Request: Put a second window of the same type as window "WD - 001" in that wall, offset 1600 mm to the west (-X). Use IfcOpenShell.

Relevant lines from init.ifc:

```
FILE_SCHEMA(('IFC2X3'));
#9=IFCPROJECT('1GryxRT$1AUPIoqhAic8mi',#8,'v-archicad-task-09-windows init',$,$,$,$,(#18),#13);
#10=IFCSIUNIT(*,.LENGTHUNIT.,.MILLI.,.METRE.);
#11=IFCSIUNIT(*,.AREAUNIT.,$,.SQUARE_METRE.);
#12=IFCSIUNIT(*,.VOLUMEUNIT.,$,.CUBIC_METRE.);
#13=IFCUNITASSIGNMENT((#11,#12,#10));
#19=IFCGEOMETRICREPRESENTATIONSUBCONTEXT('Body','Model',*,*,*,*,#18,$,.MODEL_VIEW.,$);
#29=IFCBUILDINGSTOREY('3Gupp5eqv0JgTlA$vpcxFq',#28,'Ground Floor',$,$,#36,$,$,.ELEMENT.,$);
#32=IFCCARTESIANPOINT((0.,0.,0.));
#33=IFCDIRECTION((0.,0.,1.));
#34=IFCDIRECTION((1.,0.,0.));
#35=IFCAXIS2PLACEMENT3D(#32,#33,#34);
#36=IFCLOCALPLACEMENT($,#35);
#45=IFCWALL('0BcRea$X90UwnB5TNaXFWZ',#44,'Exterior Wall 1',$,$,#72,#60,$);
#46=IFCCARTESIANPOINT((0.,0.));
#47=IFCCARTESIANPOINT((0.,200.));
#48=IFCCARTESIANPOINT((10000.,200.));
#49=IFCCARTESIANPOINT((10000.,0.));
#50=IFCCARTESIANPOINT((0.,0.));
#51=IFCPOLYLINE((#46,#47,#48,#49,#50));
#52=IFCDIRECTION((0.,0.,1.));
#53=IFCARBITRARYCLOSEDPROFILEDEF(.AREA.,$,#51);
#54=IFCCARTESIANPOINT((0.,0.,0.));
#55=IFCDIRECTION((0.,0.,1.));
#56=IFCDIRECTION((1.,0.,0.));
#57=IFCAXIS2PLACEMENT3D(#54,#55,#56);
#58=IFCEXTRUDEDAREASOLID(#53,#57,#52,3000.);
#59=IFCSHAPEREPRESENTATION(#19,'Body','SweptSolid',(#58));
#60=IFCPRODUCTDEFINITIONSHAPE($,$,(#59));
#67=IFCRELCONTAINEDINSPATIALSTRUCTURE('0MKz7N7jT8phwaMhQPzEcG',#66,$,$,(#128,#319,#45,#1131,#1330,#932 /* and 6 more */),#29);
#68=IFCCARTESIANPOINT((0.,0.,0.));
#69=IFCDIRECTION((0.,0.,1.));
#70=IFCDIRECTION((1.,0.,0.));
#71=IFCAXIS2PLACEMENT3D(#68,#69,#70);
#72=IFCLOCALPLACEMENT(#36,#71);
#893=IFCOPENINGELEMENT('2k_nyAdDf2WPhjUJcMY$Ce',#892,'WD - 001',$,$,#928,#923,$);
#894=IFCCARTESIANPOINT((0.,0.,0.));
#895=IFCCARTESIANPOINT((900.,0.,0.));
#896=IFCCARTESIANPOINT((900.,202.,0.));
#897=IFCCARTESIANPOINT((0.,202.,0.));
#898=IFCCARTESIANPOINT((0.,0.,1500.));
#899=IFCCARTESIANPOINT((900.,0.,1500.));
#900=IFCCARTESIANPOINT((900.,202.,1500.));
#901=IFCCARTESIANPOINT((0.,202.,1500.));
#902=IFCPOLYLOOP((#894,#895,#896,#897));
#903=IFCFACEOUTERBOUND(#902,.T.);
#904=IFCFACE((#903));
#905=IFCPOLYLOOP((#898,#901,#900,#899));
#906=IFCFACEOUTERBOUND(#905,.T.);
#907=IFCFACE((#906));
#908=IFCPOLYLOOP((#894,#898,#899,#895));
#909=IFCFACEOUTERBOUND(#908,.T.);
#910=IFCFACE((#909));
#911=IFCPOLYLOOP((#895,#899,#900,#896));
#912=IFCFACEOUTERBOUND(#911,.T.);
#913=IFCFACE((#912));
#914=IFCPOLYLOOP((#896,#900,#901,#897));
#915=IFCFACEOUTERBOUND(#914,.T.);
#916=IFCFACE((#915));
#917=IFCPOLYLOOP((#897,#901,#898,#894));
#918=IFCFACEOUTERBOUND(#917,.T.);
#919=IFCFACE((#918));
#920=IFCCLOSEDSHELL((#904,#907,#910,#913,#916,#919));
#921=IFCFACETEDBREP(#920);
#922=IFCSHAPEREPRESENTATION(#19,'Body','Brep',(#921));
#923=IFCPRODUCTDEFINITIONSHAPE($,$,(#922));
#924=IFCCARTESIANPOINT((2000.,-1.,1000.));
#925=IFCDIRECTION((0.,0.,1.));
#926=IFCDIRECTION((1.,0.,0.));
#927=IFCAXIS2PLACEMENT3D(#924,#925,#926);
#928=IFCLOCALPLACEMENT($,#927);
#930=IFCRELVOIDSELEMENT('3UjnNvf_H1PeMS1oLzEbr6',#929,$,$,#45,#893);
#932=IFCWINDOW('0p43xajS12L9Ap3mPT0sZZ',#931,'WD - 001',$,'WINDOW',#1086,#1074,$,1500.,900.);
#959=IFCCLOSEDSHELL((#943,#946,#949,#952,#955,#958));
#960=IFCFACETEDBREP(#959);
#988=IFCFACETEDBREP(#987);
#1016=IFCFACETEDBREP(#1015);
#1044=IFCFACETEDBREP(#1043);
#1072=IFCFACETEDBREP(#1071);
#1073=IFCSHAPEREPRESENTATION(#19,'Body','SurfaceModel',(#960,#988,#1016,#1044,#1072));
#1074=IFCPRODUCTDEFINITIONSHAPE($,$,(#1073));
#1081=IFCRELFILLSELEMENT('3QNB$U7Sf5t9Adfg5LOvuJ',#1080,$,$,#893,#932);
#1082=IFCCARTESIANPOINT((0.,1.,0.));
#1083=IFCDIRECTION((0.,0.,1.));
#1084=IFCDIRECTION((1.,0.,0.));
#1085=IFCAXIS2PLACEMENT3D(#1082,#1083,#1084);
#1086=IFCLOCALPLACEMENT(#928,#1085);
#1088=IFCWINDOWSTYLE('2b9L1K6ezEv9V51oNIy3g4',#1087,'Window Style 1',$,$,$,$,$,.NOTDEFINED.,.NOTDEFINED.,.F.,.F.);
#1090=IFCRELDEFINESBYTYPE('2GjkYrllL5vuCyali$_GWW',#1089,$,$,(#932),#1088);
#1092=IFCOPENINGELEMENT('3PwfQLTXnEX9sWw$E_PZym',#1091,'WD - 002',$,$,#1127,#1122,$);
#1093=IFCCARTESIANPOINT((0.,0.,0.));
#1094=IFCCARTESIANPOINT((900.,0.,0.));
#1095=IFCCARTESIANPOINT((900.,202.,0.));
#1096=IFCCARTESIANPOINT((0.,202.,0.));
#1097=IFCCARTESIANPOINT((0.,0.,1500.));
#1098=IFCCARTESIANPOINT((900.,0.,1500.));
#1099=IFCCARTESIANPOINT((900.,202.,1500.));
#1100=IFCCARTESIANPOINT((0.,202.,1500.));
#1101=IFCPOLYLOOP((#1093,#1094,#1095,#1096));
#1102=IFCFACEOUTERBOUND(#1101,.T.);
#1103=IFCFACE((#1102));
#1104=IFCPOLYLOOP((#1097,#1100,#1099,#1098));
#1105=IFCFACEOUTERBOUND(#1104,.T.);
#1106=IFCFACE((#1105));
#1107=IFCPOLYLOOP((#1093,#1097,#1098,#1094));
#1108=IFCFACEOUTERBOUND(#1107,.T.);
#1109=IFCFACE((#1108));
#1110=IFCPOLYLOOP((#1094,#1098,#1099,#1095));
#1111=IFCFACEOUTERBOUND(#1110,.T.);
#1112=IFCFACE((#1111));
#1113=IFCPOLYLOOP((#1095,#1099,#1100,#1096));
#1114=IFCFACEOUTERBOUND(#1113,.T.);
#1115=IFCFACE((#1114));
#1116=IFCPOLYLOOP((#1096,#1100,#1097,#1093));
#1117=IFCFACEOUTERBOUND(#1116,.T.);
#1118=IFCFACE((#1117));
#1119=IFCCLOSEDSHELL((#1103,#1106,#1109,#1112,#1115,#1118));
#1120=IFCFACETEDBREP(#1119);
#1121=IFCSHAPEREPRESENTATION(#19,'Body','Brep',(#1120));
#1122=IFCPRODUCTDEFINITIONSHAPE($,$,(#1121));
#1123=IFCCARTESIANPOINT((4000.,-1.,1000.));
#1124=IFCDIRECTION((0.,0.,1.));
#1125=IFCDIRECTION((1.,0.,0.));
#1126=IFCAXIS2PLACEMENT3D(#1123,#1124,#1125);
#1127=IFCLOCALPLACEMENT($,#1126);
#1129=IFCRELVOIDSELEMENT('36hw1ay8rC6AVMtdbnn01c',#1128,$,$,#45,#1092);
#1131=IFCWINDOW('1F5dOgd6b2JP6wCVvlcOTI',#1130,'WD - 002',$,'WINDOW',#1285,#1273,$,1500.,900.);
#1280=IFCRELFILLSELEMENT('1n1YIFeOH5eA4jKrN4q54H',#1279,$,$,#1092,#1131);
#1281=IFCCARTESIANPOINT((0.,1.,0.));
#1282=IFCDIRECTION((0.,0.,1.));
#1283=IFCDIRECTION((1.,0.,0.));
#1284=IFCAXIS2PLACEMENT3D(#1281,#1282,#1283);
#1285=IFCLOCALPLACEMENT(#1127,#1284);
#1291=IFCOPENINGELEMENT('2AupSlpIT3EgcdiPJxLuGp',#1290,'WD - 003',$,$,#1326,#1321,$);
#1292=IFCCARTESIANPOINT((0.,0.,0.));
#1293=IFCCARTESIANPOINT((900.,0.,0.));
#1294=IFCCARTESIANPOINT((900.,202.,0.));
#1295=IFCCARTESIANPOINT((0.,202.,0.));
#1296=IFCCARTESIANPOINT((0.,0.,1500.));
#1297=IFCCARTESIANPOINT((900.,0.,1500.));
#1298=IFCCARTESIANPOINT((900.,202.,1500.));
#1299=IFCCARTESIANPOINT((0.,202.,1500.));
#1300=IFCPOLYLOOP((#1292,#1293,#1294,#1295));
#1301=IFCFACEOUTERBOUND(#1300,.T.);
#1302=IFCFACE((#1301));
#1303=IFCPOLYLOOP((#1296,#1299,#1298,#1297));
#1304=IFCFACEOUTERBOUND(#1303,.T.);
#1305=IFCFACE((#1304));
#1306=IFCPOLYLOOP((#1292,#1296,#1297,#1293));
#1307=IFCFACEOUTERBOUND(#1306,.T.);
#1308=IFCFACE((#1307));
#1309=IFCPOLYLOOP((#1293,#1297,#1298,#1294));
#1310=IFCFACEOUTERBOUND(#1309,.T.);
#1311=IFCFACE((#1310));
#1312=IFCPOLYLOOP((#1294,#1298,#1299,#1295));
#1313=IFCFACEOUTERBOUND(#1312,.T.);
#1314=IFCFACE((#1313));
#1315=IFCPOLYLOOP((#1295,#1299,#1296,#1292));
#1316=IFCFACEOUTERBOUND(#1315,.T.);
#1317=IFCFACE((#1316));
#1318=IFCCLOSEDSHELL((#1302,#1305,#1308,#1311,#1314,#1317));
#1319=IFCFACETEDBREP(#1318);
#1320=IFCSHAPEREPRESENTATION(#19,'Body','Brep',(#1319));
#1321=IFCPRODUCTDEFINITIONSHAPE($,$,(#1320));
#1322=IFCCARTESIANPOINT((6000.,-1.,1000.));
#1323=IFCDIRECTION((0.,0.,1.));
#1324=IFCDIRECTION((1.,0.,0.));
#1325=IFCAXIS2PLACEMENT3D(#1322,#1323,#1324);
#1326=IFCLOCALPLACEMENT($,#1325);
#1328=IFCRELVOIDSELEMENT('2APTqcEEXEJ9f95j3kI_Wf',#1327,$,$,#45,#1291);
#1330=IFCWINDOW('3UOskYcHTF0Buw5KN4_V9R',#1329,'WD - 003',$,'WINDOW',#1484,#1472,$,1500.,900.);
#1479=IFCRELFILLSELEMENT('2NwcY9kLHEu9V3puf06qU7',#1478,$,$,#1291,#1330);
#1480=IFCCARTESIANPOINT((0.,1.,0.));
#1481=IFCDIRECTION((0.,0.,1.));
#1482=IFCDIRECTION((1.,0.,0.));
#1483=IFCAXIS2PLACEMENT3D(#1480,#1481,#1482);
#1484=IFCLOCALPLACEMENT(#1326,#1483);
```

```python
import ifcopenshell
import ifcopenshell.api.feature
import ifcopenshell.api.geometry
import ifcopenshell.api.root
import ifcopenshell.geom
import ifcopenshell.util.element
import ifcopenshell.util.placement
import ifcopenshell.util.shape
import ifcopenshell.util.unit

model = ifcopenshell.open("init.ifc")
unit_scale = ifcopenshell.util.unit.calculate_unit_scale(model)
settings = ifcopenshell.geom.settings()


def volume(element):
    """Net volume in cubic metres, openings subtracted."""
    shape = ifcopenshell.geom.create_shape(settings, element)
    return ifcopenshell.util.shape.get_volume(shape.geometry)


window = model.by_guid("0p43xajS12L9Ap3mPT0sZZ")
opening = window.FillsVoids[0].RelatingOpeningElement
wall = opening.VoidsElements[0].RelatingBuildingElement
before = volume(wall)
shift = ifcopenshell.util.placement.get_local_placement(wall.ObjectPlacement)[:3, 0] * -1.6 / unit_scale

# copy_class copies the void relationship, type, container and properties, but no geometry.
new_opening = ifcopenshell.api.root.copy_class(model, product=opening)
new_opening.Representation = ifcopenshell.util.element.copy_deep(
    model, opening.Representation, exclude=["IfcGeometricRepresentationContext", "IfcRepresentationMap"]
)
new_window = ifcopenshell.api.root.copy_class(model, product=window)
new_window.Representation = ifcopenshell.util.element.copy_deep(
    model, window.Representation, exclude=["IfcGeometricRepresentationContext", "IfcRepresentationMap"]
)
fills = ifcopenshell.api.feature.add_filling(model, opening=new_opening, element=new_window)
fills.OwnerHistory = new_window.OwnerHistory  # required in IFC2X3

for old, new in ((opening, new_opening), (window, new_window)):
    matrix = ifcopenshell.util.placement.get_local_placement(old.ObjectPlacement)
    matrix[:3, 3] += shift
    ifcopenshell.api.geometry.edit_object_placement(model, product=new, matrix=matrix, is_si=False)

after = volume(wall)

print(f"wall volume {before:.3f} -> {after:.3f} m3")

model.write("init_rev.ifc")
```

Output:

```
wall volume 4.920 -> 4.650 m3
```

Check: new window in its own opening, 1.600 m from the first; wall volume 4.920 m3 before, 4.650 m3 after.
